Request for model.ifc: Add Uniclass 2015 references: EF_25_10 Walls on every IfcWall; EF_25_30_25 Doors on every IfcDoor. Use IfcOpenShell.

First a look at what the model holds.

```python
import ifcopenshell

model = ifcopenshell.open("model.ifc")
print(model.schema)
print("classifications:", [c.Name for c in model.by_type("IfcClassification")])
for ifc_class in ("IfcDoor", "IfcRoof", "IfcStair", "IfcWall", "IfcWindow"):
    print(ifc_class, len(model.by_type(ifc_class)))
```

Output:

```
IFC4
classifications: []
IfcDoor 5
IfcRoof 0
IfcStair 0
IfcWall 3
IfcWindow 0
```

```python
import ifcopenshell
import ifcopenshell.api.classification

model = ifcopenshell.open("model.ifc")

system = ifcopenshell.api.classification.add_classification(model, classification="Uniclass 2015")

codes = {
    "IfcWall": ("EF_25_10", "Walls"),
    "IfcDoor": ("EF_25_30_25", "Doors"),
}
for ifc_class, (code, name) in codes.items():
    products = model.by_type(ifc_class)
    ifcopenshell.api.classification.add_reference(
        model, products=products, classification=system, identification=code, name=name
    )
    print(code, len(products))

model.write("model_updated.ifc")
```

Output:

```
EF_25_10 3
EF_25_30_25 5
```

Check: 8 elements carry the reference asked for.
